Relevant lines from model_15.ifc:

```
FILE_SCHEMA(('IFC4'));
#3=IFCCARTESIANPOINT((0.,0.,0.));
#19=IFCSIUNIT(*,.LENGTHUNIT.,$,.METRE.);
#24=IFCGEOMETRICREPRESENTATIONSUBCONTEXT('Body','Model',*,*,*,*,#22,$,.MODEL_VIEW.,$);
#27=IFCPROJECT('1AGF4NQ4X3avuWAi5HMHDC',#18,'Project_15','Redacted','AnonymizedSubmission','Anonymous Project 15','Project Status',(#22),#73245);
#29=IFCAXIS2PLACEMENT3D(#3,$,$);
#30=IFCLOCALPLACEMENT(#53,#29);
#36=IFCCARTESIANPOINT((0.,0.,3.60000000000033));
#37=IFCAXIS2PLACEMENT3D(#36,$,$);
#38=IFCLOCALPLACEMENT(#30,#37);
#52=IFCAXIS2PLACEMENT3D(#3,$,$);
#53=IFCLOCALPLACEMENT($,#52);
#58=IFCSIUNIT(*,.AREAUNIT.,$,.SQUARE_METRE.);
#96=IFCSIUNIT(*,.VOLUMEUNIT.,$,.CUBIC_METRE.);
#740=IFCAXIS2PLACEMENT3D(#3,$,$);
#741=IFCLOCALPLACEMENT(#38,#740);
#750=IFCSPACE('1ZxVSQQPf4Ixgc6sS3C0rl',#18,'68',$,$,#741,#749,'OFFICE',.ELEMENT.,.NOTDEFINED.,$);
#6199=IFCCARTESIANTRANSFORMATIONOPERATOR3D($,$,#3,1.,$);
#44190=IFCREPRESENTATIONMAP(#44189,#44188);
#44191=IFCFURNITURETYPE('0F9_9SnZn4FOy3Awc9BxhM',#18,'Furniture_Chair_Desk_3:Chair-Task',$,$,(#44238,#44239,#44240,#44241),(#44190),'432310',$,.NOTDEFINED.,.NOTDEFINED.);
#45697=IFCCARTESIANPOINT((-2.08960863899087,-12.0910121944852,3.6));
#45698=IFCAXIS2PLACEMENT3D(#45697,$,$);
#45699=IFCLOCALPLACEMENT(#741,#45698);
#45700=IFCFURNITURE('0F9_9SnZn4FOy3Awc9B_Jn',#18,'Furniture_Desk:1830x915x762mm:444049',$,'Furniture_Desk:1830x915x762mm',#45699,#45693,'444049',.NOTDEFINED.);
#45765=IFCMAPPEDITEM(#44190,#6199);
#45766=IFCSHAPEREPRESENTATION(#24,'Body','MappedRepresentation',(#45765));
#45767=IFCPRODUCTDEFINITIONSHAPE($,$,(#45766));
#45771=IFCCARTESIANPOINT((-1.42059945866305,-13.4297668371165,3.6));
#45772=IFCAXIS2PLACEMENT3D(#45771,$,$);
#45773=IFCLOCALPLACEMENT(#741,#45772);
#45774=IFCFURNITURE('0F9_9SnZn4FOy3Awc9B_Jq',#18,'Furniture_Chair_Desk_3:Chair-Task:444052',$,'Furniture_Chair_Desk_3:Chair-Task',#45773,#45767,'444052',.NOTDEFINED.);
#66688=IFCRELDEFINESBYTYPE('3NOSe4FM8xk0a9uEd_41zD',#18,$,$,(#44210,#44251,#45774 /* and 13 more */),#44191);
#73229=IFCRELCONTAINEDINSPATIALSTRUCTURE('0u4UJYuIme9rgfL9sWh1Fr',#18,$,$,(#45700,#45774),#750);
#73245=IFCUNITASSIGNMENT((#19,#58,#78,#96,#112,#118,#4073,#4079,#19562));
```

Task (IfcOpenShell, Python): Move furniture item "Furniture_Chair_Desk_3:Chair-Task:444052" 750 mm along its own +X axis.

```python
import ifcopenshell
import ifcopenshell.api.geometry
import ifcopenshell.util.placement

model = ifcopenshell.open("model_15.ifc")

item = model.by_guid("0F9_9SnZn4FOy3Awc9B_Jq")
matrix = ifcopenshell.util.placement.get_local_placement(item.ObjectPlacement)
matrix[:3, 3] += matrix[:3, 0] * 0.75
ifcopenshell.api.geometry.edit_object_placement(model, product=item, matrix=matrix, is_si=False)

print(ifcopenshell.util.placement.get_local_placement(item.ObjectPlacement).round(3) + 0.0)

model.write("model_15-out.ifc")
```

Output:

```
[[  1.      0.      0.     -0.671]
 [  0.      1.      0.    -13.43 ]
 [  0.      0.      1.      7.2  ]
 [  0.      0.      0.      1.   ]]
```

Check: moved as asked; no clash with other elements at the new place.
